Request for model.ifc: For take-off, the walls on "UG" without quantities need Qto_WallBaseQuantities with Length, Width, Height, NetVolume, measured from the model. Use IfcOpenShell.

First a look at what the model holds.

```python
import ifcopenshell
import ifcopenshell.util.element
import ifcopenshell.util.unit

model = ifcopenshell.open("model.ifc")
print(model.schema)
for unit_type in ("LENGTHUNIT", "AREAUNIT", "VOLUMEUNIT"):
    print(unit_type, ifcopenshell.util.unit.calculate_unit_scale(model, unit_type))
storey = next(s for s in model.by_type("IfcBuildingStorey") if s.Name == "UG")
walls = [e for e in ifcopenshell.util.element.get_decomposition(storey) if e.is_a("IfcWall")]
for e in sorted(walls, key=lambda e: e.id()):
    print(e.id(), e.is_a(), e.Name, list(ifcopenshell.util.element.get_psets(e, qtos_only=True)), sep=" | ")
```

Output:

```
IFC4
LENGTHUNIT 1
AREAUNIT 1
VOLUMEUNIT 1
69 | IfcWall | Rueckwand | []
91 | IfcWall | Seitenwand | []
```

```python
import ifcopenshell
import ifcopenshell.api.pset
import ifcopenshell.geom
import ifcopenshell.util.element
import ifcopenshell.util.shape
import ifcopenshell.util.unit

model = ifcopenshell.open("model.ifc")
unit_scale = ifcopenshell.util.unit.calculate_unit_scale(model)
volume_scale = ifcopenshell.util.unit.calculate_unit_scale(model, "VOLUMEUNIT")
settings = ifcopenshell.geom.settings()

storey = next(s for s in model.by_type("IfcBuildingStorey") if s.Name == "UG")
walls = [e for e in ifcopenshell.util.element.get_decomposition(storey) if e.is_a("IfcWall")]

for e in sorted(walls, key=lambda e: e.id()):
    if ifcopenshell.util.element.get_psets(e, qtos_only=True, should_inherit=False):
        continue
    # Geometry comes back in metres, in the element's own axes.
    shape = ifcopenshell.geom.create_shape(settings, e)
    values = {
        "Length": ifcopenshell.util.shape.get_x(shape.geometry) / unit_scale,
        "Width": ifcopenshell.util.shape.get_y(shape.geometry) / unit_scale,
        "Height": ifcopenshell.util.shape.get_z(shape.geometry) / unit_scale,
        "NetVolume": ifcopenshell.util.shape.get_volume(shape.geometry) / volume_scale,
    }
    qto = ifcopenshell.api.pset.add_qto(model, product=e, name="Qto_WallBaseQuantities")
    ifcopenshell.api.pset.edit_qto(model, qto=qto, properties=values)
    print(e.id(), {k: round(v, 3) for k, v in values.items()})

model.write("model_edited.ifc")
```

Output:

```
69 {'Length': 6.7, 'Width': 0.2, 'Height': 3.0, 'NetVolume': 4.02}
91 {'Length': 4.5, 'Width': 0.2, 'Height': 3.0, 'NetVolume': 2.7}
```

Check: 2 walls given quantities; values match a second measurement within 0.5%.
